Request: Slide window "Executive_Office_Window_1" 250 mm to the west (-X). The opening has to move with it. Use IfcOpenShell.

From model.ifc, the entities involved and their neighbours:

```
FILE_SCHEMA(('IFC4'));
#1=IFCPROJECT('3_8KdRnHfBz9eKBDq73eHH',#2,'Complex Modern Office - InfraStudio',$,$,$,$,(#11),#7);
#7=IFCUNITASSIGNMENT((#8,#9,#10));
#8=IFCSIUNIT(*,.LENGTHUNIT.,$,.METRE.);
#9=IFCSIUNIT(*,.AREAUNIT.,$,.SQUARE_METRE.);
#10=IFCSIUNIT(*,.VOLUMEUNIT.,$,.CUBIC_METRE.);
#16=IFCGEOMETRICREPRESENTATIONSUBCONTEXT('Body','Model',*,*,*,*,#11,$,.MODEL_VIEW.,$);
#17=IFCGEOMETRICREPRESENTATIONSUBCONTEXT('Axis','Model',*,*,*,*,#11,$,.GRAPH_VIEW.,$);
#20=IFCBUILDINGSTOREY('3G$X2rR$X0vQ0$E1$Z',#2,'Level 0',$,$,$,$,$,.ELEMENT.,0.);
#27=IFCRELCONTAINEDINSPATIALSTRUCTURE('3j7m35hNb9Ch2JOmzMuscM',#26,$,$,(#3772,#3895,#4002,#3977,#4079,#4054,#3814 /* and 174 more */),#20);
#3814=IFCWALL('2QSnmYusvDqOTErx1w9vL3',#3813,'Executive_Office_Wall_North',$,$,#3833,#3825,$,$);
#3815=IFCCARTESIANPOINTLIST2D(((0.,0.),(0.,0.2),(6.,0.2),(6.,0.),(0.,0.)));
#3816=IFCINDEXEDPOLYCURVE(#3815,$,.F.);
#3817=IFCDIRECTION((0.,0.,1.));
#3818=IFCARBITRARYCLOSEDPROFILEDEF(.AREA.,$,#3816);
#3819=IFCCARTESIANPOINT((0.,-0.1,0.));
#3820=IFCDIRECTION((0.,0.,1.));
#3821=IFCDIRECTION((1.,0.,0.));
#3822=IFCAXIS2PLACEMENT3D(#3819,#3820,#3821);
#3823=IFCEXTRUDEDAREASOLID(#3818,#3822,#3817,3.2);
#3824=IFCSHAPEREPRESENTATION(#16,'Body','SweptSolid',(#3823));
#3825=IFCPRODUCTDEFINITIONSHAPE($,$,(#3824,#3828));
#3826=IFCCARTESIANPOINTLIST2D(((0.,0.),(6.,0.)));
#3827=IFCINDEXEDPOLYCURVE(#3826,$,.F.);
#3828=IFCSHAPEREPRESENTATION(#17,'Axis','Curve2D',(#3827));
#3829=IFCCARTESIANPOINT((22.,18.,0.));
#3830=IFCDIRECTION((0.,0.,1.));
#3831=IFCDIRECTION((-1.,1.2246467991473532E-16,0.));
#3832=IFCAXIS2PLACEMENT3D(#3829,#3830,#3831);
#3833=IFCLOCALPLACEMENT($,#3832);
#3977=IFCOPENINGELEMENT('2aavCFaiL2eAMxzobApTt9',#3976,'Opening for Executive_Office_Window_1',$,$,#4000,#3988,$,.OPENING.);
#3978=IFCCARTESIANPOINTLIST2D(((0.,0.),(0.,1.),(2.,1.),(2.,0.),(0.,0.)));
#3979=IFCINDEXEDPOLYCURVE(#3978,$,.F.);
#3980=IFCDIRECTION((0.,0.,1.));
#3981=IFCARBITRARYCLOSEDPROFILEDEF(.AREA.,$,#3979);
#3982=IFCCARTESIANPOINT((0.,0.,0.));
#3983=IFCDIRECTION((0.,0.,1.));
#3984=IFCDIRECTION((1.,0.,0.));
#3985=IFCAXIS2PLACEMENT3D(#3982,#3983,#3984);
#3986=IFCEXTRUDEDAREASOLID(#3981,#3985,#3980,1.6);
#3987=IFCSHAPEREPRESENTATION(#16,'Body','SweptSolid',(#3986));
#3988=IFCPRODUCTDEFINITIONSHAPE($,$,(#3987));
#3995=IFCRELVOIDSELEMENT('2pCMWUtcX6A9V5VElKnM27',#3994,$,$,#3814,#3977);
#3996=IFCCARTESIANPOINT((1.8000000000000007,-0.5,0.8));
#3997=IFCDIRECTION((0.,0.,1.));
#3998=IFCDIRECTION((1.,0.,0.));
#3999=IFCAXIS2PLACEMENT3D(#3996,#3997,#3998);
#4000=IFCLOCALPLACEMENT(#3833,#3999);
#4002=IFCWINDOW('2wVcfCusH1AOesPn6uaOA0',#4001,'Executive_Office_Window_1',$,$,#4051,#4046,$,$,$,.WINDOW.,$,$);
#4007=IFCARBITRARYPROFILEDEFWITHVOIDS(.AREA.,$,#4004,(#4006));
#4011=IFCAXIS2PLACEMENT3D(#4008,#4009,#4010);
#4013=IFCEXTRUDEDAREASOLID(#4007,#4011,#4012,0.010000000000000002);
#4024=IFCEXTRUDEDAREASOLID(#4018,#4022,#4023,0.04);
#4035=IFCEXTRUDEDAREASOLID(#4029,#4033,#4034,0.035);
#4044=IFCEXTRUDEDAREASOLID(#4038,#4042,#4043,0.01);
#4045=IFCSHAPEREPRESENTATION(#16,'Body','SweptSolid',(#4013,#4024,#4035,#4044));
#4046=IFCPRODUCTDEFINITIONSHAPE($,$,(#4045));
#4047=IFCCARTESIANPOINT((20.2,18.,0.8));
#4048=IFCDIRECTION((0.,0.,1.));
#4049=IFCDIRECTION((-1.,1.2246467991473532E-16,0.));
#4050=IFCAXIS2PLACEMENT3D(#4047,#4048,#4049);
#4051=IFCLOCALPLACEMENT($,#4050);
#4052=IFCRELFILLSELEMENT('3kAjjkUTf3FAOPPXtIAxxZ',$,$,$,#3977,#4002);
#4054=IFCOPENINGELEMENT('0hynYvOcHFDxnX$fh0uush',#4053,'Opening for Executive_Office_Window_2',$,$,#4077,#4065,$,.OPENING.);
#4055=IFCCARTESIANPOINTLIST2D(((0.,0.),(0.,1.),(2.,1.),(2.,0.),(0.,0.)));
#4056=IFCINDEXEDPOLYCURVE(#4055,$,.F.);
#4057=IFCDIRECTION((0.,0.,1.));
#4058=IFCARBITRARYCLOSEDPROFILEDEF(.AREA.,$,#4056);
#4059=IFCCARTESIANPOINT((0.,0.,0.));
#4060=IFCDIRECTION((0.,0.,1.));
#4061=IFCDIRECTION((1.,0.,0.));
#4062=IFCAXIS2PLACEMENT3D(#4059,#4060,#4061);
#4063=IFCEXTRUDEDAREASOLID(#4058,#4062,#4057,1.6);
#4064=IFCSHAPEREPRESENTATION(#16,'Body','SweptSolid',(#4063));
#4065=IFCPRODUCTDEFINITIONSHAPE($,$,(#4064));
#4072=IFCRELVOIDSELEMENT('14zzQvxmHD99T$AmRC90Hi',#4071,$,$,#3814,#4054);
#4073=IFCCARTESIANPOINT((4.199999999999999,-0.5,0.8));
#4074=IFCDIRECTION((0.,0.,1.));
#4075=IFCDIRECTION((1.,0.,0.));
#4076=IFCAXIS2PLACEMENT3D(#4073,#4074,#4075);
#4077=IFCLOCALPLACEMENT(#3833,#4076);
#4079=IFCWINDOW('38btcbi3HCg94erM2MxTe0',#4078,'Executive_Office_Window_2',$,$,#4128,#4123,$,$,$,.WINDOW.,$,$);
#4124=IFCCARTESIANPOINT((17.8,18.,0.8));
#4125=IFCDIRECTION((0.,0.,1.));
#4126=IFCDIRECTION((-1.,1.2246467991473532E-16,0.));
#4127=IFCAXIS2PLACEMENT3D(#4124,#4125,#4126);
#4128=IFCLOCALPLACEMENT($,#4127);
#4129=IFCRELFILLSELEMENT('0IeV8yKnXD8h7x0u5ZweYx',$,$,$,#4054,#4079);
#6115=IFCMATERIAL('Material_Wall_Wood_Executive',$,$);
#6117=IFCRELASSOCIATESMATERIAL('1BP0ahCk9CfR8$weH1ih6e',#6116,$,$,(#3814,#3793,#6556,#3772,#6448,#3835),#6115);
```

```python
import ifcopenshell
import ifcopenshell.api.geometry
import ifcopenshell.util.placement
import ifcopenshell.util.unit

model = ifcopenshell.open("model.ifc")
unit_scale = ifcopenshell.util.unit.calculate_unit_scale(model)

window = model.by_guid("2wVcfCusH1AOesPn6uaOA0")
opening = window.FillsVoids[0].RelatingOpeningElement
wall = opening.VoidsElements[0].RelatingBuildingElement

wall_matrix = ifcopenshell.util.placement.get_local_placement(wall.ObjectPlacement)
shift = wall_matrix[:3, 0] * 0.25 / unit_scale
before = ifcopenshell.util.placement.get_local_placement(window.ObjectPlacement)[:3, 3].copy()

# The window is not placed relative to its opening, so move both.
for product in (opening, window):
    matrix = ifcopenshell.util.placement.get_local_placement(product.ObjectPlacement)
    matrix[:3, 3] += shift
    ifcopenshell.api.geometry.edit_object_placement(model, product=product, matrix=matrix, is_si=False)

after = ifcopenshell.util.placement.get_local_placement(window.ObjectPlacement)[:3, 3]
print("window moved by", (after - before).round(3) + 0.0)

model.write("model-out.ifc")
```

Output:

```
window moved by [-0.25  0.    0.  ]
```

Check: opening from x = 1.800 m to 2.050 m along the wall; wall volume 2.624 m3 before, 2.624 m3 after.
